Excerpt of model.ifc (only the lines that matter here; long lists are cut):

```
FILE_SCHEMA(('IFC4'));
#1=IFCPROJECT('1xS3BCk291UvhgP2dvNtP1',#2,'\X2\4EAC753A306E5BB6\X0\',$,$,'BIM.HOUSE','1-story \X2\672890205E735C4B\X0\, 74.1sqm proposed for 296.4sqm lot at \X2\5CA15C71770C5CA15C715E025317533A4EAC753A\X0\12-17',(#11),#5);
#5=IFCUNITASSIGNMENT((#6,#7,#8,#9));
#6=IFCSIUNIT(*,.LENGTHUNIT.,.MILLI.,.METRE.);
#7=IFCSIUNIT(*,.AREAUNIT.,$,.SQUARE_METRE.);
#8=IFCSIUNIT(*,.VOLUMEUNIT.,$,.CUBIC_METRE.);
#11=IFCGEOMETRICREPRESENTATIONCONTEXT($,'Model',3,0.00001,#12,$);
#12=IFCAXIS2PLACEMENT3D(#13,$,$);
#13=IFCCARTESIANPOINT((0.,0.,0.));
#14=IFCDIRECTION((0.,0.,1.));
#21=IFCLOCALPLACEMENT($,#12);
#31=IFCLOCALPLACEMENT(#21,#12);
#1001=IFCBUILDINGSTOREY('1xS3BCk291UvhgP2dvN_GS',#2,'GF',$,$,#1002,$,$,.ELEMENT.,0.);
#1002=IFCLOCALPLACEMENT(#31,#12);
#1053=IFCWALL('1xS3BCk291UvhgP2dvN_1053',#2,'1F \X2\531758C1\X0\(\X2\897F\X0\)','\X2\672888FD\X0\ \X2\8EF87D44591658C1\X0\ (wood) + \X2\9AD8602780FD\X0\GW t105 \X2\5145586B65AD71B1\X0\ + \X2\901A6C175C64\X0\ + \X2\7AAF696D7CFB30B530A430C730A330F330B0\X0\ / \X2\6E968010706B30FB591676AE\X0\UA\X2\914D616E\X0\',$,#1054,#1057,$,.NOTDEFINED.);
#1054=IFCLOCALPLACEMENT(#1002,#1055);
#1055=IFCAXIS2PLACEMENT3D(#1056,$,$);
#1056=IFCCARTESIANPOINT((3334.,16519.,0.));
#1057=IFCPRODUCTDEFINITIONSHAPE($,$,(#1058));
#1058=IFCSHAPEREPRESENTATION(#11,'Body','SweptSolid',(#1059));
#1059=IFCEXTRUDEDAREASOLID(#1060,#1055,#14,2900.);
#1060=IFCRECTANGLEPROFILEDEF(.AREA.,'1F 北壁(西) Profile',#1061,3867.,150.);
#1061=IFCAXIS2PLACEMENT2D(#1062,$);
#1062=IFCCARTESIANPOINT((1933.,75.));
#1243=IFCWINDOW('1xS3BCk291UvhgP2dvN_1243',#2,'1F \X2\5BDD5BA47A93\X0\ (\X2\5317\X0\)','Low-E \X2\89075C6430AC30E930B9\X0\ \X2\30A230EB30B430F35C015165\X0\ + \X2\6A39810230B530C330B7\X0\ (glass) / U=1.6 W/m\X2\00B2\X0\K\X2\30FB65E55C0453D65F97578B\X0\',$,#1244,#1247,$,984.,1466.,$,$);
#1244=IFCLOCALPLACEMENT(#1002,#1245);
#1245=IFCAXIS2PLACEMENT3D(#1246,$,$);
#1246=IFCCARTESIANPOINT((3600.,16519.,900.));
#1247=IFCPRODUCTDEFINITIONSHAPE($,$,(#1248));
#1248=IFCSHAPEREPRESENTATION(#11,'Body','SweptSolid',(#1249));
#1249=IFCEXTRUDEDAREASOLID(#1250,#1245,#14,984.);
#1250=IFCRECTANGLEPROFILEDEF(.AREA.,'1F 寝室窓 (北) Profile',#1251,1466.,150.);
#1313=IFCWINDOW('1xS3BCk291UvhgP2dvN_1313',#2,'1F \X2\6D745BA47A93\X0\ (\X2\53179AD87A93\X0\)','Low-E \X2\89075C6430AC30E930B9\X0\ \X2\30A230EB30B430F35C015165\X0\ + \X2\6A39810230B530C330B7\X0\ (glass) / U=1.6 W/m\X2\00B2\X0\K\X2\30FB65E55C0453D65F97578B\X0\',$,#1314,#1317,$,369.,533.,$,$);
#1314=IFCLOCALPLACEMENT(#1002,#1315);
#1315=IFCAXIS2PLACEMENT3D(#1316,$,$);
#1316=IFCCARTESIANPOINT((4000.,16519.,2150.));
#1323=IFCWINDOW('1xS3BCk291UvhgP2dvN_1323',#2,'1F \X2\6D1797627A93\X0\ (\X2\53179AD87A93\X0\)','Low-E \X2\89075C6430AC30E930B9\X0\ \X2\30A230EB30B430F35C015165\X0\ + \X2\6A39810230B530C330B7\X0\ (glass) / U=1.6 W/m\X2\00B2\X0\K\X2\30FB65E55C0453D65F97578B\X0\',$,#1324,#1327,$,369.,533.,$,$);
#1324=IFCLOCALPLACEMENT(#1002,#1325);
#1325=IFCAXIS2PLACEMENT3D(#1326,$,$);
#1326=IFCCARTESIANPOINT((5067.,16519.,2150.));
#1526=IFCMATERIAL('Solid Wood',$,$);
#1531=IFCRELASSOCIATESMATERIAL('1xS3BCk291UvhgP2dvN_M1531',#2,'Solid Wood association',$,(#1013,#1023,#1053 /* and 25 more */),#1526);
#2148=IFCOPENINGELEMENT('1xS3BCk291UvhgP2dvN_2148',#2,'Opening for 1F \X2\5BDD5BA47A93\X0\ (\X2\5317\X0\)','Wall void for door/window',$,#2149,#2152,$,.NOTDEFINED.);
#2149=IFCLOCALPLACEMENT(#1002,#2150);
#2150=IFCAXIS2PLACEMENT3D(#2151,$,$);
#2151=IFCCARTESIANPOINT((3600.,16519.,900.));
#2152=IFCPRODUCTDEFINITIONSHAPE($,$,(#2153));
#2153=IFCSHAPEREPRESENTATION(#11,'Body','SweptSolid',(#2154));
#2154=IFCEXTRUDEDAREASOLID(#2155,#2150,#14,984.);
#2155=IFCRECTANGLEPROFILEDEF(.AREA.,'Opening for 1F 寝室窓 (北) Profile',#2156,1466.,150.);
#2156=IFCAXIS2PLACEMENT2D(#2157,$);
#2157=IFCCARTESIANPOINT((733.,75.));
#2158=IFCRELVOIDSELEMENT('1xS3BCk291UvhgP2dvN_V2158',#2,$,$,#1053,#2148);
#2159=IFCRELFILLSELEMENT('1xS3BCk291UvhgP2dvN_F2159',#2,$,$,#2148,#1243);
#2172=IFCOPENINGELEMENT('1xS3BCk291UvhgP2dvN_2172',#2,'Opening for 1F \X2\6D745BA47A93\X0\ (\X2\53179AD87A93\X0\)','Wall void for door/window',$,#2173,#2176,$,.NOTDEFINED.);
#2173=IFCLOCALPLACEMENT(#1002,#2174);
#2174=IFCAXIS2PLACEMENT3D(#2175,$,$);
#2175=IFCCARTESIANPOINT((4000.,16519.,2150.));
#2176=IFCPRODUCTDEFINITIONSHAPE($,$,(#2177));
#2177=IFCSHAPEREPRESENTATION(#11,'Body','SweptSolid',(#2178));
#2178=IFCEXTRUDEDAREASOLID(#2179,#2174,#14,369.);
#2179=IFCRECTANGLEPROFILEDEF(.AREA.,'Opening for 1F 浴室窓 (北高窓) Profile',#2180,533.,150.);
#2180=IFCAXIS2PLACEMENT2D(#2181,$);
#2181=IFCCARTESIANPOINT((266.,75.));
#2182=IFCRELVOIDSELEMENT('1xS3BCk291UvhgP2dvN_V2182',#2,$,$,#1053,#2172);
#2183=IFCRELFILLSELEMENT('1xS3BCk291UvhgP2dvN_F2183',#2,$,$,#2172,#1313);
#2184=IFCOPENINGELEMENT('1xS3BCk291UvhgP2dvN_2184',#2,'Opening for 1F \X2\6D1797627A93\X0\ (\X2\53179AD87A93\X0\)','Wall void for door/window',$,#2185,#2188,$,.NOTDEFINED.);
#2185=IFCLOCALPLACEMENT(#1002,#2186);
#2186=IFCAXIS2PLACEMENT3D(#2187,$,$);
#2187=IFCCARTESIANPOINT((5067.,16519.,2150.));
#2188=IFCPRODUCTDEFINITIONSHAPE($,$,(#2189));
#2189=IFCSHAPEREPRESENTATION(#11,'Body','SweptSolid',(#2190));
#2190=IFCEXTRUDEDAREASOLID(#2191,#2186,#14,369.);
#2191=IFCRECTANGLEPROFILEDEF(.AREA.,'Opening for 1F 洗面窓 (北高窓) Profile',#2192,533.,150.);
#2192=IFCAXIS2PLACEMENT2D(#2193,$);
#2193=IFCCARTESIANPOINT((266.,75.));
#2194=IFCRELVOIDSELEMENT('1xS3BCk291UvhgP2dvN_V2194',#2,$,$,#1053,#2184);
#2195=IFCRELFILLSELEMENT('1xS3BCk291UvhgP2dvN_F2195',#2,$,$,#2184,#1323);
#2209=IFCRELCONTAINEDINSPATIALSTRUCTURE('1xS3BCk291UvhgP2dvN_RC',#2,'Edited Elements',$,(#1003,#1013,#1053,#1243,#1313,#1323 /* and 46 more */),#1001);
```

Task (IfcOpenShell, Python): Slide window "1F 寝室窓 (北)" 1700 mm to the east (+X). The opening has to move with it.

```python
import ifcopenshell
import ifcopenshell.api.geometry
import ifcopenshell.util.placement
import ifcopenshell.util.unit

model = ifcopenshell.open("model.ifc")
unit_scale = ifcopenshell.util.unit.calculate_unit_scale(model)

window = model.by_guid("1xS3BCk291UvhgP2dvN_1243")
opening = window.FillsVoids[0].RelatingOpeningElement
wall = opening.VoidsElements[0].RelatingBuildingElement

wall_matrix = ifcopenshell.util.placement.get_local_placement(wall.ObjectPlacement)
shift = wall_matrix[:3, 0] * 1.7 / unit_scale
before = ifcopenshell.util.placement.get_local_placement(window.ObjectPlacement)[:3, 3].copy()

# The window is not placed relative to its opening, so move both.
for product in (opening, window):
    matrix = ifcopenshell.util.placement.get_local_placement(product.ObjectPlacement)
    matrix[:3, 3] += shift
    ifcopenshell.api.geometry.edit_object_placement(model, product=product, matrix=matrix, is_si=False)

after = ifcopenshell.util.placement.get_local_placement(window.ObjectPlacement)[:3, 3]
print("window moved by", (after - before).round(3) + 0.0)

model.write("model_v2.ifc")
```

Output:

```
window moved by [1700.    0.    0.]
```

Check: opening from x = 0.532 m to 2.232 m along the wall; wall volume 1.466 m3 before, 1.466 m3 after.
